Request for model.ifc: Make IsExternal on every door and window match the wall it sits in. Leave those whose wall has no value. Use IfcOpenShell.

First a look at what the model holds.

```python
import ifcopenshell
import ifcopenshell.util.element

model = ifcopenshell.open("model.ifc")
print(model.schema)
seen = {}
for e in model.by_type("IfcDoor") + model.by_type("IfcWindow"):
    if not e.FillsVoids:
        continue
    host = e.FillsVoids[0].RelatingOpeningElement.VoidsElements[0].RelatingBuildingElement
    own = ifcopenshell.util.element.get_pset(e, f"Pset_{e.is_a()[3:].removesuffix('StandardCase')}Common", "IsExternal")
    wall = ifcopenshell.util.element.get_pset(host, "Pset_WallCommon", "IsExternal")
    seen[e.is_a(), own, wall] = seen.get((e.is_a(), own, wall), 0) + 1
for (cls, own, wall), count in sorted(seen.items(), key=str):
    print(count, cls, "IsExternal:", own, "| host wall:", wall)
```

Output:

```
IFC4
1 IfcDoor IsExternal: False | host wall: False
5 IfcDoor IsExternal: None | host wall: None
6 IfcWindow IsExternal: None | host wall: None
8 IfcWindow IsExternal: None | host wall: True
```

```python
import ifcopenshell
import ifcopenshell.api.pset
import ifcopenshell.util.element

model = ifcopenshell.open("model.ifc")

count = 0
for ifc_class, pset_name in (("IfcDoor", "Pset_DoorCommon"), ("IfcWindow", "Pset_WindowCommon")):
    for e in model.by_type(ifc_class):
        if not e.FillsVoids:
            continue
        host = e.FillsVoids[0].RelatingOpeningElement.VoidsElements[0].RelatingBuildingElement
        external = ifcopenshell.util.element.get_pset(host, "Pset_WallCommon", "IsExternal")
        if external is None or ifcopenshell.util.element.get_pset(e, pset_name, "IsExternal") == external:
            continue
        pset = ifcopenshell.api.pset.add_pset(model, product=e, name=pset_name)
        ifcopenshell.api.pset.edit_pset(model, pset=pset, properties={"IsExternal": external})
        count += 1

print(count, "updated")

model.write("model_v2.ifc")
```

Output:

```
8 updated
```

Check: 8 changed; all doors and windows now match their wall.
